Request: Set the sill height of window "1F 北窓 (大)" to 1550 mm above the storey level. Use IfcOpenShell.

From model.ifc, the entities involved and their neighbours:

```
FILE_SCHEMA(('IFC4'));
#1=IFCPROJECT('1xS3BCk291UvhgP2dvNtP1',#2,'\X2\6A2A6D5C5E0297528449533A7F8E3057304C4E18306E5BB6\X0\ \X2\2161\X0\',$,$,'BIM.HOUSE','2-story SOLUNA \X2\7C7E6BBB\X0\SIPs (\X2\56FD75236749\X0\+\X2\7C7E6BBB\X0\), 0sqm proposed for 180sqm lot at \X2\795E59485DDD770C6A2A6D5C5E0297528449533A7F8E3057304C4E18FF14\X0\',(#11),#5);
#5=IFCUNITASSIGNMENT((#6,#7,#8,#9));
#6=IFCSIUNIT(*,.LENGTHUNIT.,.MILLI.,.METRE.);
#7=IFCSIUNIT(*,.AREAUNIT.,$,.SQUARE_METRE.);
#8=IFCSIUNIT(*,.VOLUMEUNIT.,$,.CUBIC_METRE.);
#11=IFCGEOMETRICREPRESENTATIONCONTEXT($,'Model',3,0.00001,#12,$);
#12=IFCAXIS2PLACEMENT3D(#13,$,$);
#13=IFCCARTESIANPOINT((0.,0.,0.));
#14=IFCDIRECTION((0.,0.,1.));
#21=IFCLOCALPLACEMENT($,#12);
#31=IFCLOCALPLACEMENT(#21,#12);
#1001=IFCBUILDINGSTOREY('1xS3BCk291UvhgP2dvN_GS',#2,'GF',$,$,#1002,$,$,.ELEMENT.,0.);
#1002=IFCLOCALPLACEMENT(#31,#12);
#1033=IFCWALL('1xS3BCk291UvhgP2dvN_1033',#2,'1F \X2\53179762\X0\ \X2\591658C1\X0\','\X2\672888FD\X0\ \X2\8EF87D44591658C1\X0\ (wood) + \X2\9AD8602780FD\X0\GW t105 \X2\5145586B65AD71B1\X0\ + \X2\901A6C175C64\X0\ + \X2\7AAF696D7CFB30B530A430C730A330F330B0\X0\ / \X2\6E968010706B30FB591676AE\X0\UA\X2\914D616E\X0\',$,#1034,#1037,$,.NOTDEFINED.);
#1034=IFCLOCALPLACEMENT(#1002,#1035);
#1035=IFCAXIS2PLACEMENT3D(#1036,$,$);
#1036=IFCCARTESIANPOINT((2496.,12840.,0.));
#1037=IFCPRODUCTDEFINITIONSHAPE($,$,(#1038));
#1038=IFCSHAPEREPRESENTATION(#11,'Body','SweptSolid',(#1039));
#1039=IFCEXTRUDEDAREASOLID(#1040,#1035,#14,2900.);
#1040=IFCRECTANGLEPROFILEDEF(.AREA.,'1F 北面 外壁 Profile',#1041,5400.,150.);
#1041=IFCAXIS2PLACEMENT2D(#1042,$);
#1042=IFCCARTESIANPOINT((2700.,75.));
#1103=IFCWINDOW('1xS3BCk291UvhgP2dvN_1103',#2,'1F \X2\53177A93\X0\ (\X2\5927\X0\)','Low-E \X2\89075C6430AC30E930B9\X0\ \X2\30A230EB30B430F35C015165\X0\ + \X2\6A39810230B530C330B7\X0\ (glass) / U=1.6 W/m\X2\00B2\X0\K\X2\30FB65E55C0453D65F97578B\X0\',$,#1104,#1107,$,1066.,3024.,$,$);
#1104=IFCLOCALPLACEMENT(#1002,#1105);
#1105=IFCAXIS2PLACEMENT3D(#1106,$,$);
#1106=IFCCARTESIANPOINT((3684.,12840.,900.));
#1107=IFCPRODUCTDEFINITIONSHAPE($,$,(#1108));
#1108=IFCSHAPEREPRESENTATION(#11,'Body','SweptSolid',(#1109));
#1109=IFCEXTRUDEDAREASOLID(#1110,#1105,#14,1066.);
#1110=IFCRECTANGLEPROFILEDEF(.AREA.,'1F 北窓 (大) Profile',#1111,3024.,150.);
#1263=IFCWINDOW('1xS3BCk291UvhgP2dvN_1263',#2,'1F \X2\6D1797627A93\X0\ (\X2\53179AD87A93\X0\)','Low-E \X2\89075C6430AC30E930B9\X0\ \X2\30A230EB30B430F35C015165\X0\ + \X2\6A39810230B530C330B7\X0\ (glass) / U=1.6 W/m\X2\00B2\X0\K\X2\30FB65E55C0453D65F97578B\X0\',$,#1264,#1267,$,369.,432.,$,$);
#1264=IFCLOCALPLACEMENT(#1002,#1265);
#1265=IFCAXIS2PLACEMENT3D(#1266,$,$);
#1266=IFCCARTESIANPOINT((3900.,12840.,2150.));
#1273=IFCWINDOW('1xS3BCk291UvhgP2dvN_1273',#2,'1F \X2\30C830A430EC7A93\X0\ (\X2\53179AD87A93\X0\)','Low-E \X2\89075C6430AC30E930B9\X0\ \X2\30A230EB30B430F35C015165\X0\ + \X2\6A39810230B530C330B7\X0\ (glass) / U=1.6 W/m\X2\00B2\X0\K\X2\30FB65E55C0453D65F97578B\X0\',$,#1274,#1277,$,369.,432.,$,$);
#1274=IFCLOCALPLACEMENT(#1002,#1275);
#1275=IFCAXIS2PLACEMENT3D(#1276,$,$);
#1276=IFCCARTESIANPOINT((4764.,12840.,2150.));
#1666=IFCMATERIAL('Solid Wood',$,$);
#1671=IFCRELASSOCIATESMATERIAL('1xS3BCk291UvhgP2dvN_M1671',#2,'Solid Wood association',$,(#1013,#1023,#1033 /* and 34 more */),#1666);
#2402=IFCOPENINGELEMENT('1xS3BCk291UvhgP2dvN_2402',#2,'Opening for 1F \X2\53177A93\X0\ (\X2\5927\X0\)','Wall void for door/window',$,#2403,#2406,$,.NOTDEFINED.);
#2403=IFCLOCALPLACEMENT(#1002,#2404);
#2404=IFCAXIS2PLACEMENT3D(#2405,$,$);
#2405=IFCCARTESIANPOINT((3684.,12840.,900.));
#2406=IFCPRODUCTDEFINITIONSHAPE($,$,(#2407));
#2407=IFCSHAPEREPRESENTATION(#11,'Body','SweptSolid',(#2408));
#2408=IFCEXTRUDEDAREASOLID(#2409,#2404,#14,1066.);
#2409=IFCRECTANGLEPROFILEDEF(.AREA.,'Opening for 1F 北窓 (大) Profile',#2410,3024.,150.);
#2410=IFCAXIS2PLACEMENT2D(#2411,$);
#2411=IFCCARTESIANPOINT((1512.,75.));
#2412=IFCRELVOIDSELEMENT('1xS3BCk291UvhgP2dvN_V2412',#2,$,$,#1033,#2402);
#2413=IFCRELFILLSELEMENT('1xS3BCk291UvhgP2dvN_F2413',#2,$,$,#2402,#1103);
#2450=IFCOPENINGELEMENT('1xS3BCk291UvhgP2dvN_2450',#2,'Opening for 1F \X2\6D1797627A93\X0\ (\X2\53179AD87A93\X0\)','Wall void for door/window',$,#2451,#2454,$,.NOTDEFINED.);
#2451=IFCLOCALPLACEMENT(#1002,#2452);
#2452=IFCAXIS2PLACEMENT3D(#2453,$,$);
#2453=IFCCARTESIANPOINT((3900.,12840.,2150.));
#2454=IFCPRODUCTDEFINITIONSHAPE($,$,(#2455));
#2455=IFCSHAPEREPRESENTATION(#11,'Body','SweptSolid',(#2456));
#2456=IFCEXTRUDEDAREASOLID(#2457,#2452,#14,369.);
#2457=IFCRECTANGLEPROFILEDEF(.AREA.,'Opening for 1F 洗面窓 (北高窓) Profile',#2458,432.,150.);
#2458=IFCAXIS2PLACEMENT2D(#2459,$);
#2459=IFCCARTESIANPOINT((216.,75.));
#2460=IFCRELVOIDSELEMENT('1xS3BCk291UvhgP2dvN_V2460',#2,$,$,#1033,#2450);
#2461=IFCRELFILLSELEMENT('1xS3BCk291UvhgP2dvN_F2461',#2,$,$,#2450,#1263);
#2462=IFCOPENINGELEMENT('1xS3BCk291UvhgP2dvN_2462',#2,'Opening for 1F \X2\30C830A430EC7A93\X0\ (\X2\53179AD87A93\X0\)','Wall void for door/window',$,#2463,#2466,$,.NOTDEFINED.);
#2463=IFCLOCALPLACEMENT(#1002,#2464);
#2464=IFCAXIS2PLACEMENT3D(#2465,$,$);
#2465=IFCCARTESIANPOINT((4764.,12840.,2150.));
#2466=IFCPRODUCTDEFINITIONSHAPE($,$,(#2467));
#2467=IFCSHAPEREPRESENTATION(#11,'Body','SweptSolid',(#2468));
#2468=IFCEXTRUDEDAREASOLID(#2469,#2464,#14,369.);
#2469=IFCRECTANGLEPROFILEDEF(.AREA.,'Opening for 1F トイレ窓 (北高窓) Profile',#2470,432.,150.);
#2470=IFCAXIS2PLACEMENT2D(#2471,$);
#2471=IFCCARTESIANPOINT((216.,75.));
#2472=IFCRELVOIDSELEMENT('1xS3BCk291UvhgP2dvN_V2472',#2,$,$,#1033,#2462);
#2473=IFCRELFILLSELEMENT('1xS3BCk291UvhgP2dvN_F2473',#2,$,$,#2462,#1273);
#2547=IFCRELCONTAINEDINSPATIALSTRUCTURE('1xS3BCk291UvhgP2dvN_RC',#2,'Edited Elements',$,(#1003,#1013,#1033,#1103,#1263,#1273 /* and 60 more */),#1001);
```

```python
import numpy as np
import ifcopenshell
import ifcopenshell.api.geometry
import ifcopenshell.geom
import ifcopenshell.util.element
import ifcopenshell.util.placement
import ifcopenshell.util.shape
import ifcopenshell.util.unit

model = ifcopenshell.open("model.ifc")
unit_scale = ifcopenshell.util.unit.calculate_unit_scale(model)

window = model.by_guid("1xS3BCk291UvhgP2dvN_1103")
opening = window.FillsVoids[0].RelatingOpeningElement
storey = ifcopenshell.util.element.get_container(window, ifc_class="IfcBuildingStorey")
level = ifcopenshell.util.placement.get_local_placement(storey.ObjectPlacement)[2, 3]

# The opening's origin need not be at the sill, so measure its lowest point.
shape = ifcopenshell.geom.create_shape(ifcopenshell.geom.settings(), opening)
bottom = ifcopenshell.util.shape.get_shape_bottom_elevation(shape, shape.geometry) / unit_scale
dz = level + 1550.0 - bottom

shift = np.array([0.0, 0.0, dz])
# The window is not placed relative to its opening, so move both.
for product in (opening, window):
    matrix = ifcopenshell.util.placement.get_local_placement(product.ObjectPlacement)
    matrix[:3, 3] += shift
    ifcopenshell.api.geometry.edit_object_placement(model, product=product, matrix=matrix, is_si=False)

print(f"moved by {dz * unit_scale:+.3f} m")

model.write("model_rev.ifc")
```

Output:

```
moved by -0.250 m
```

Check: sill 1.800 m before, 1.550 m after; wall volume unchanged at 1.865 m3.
